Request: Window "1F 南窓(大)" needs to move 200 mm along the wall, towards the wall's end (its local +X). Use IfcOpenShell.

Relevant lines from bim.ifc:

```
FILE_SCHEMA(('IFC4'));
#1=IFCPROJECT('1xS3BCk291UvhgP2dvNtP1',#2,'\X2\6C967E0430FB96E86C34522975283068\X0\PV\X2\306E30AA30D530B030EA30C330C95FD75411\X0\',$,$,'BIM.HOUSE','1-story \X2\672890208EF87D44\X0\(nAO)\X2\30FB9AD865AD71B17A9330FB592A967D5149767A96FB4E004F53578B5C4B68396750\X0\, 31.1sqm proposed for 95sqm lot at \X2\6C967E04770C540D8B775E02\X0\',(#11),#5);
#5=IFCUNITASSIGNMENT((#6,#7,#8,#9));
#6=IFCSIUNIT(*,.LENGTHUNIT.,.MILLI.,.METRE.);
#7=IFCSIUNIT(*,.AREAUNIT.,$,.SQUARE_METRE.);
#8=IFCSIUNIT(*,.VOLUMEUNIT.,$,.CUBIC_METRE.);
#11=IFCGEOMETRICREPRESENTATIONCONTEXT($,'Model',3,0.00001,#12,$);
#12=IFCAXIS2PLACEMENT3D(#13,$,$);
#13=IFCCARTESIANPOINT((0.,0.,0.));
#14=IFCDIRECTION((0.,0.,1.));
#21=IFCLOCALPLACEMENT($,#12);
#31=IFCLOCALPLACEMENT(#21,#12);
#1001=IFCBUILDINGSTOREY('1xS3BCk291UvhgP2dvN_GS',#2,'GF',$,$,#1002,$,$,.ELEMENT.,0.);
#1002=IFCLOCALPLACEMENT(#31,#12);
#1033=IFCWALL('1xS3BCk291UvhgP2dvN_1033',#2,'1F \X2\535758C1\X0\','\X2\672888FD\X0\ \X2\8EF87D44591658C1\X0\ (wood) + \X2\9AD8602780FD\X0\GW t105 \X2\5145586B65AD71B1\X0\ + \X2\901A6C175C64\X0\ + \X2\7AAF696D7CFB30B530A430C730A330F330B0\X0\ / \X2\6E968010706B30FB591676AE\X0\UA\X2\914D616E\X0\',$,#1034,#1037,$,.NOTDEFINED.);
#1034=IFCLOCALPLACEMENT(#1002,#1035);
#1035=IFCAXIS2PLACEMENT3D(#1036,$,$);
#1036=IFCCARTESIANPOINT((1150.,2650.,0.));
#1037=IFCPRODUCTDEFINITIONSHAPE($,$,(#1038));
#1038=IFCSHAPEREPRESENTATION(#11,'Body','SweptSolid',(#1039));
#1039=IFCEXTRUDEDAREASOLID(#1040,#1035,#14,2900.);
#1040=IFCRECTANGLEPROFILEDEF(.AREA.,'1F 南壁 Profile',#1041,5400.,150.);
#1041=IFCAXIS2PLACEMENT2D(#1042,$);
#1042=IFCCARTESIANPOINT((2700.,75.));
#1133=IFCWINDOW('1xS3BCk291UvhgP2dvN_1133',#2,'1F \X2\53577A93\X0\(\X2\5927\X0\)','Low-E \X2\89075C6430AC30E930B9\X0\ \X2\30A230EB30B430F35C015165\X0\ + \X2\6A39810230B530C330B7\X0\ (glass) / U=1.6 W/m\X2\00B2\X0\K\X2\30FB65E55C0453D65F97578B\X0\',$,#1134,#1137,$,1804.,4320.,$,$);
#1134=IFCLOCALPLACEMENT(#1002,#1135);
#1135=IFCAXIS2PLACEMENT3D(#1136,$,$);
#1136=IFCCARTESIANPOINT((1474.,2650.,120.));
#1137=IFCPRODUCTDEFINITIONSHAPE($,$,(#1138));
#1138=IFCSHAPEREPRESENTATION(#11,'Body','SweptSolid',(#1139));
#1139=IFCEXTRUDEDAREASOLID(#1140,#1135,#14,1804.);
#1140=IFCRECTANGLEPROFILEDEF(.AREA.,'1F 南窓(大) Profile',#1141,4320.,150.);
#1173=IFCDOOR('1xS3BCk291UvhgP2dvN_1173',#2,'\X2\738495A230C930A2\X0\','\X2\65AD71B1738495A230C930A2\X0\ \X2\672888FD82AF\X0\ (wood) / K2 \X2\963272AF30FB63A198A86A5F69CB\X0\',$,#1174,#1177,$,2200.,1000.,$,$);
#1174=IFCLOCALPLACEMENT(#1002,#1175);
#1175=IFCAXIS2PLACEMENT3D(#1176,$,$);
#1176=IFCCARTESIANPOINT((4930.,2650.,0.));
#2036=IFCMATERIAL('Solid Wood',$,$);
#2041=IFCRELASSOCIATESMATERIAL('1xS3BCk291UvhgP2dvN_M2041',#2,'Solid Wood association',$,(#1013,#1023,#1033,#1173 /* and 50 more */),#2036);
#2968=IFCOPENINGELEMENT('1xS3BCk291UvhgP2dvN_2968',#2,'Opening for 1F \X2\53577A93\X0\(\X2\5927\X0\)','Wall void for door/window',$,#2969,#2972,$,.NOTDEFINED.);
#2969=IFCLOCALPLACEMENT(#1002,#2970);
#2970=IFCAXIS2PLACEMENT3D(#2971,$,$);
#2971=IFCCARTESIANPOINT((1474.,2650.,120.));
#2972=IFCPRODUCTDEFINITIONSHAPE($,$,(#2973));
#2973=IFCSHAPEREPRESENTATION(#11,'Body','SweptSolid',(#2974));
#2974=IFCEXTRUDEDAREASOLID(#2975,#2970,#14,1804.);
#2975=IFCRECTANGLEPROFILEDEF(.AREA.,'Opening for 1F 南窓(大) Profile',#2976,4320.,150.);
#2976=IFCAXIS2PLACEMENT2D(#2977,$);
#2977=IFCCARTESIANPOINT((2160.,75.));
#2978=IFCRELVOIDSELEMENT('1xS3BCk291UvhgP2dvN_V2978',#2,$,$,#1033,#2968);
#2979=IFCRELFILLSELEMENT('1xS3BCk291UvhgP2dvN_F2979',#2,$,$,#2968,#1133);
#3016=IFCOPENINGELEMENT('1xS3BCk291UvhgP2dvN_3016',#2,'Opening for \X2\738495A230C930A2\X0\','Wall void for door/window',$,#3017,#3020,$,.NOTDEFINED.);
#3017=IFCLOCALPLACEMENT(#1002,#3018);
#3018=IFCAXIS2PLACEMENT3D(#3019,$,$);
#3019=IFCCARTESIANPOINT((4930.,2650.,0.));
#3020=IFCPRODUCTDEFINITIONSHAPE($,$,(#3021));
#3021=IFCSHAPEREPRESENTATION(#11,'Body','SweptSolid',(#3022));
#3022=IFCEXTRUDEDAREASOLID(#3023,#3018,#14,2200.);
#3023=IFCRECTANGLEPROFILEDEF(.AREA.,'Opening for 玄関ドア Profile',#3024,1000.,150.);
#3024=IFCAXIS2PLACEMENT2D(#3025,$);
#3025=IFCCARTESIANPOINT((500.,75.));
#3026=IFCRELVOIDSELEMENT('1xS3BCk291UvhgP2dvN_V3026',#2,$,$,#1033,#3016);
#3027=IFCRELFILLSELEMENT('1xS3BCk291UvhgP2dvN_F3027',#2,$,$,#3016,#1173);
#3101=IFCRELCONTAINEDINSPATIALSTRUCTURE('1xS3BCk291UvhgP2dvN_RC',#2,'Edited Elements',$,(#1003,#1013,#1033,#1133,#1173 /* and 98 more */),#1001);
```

```python
import ifcopenshell
import ifcopenshell.api.geometry
import ifcopenshell.util.placement
import ifcopenshell.util.unit

model = ifcopenshell.open("bim.ifc")
unit_scale = ifcopenshell.util.unit.calculate_unit_scale(model)

window = model.by_guid("1xS3BCk291UvhgP2dvN_1133")
opening = window.FillsVoids[0].RelatingOpeningElement
wall = opening.VoidsElements[0].RelatingBuildingElement

wall_matrix = ifcopenshell.util.placement.get_local_placement(wall.ObjectPlacement)
shift = wall_matrix[:3, 0] * 0.2 / unit_scale
before = ifcopenshell.util.placement.get_local_placement(window.ObjectPlacement)[:3, 3].copy()

# The window is not placed relative to its opening, so move both.
for product in (opening, window):
    matrix = ifcopenshell.util.placement.get_local_placement(product.ObjectPlacement)
    matrix[:3, 3] += shift
    ifcopenshell.api.geometry.edit_object_placement(model, product=product, matrix=matrix, is_si=False)

after = ifcopenshell.util.placement.get_local_placement(window.ObjectPlacement)[:3, 3]
print("window moved by", (after - before).round(3) + 0.0)

model.write("bim_rev.ifc")
```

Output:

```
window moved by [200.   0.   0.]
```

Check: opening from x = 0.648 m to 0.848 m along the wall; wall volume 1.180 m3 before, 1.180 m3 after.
